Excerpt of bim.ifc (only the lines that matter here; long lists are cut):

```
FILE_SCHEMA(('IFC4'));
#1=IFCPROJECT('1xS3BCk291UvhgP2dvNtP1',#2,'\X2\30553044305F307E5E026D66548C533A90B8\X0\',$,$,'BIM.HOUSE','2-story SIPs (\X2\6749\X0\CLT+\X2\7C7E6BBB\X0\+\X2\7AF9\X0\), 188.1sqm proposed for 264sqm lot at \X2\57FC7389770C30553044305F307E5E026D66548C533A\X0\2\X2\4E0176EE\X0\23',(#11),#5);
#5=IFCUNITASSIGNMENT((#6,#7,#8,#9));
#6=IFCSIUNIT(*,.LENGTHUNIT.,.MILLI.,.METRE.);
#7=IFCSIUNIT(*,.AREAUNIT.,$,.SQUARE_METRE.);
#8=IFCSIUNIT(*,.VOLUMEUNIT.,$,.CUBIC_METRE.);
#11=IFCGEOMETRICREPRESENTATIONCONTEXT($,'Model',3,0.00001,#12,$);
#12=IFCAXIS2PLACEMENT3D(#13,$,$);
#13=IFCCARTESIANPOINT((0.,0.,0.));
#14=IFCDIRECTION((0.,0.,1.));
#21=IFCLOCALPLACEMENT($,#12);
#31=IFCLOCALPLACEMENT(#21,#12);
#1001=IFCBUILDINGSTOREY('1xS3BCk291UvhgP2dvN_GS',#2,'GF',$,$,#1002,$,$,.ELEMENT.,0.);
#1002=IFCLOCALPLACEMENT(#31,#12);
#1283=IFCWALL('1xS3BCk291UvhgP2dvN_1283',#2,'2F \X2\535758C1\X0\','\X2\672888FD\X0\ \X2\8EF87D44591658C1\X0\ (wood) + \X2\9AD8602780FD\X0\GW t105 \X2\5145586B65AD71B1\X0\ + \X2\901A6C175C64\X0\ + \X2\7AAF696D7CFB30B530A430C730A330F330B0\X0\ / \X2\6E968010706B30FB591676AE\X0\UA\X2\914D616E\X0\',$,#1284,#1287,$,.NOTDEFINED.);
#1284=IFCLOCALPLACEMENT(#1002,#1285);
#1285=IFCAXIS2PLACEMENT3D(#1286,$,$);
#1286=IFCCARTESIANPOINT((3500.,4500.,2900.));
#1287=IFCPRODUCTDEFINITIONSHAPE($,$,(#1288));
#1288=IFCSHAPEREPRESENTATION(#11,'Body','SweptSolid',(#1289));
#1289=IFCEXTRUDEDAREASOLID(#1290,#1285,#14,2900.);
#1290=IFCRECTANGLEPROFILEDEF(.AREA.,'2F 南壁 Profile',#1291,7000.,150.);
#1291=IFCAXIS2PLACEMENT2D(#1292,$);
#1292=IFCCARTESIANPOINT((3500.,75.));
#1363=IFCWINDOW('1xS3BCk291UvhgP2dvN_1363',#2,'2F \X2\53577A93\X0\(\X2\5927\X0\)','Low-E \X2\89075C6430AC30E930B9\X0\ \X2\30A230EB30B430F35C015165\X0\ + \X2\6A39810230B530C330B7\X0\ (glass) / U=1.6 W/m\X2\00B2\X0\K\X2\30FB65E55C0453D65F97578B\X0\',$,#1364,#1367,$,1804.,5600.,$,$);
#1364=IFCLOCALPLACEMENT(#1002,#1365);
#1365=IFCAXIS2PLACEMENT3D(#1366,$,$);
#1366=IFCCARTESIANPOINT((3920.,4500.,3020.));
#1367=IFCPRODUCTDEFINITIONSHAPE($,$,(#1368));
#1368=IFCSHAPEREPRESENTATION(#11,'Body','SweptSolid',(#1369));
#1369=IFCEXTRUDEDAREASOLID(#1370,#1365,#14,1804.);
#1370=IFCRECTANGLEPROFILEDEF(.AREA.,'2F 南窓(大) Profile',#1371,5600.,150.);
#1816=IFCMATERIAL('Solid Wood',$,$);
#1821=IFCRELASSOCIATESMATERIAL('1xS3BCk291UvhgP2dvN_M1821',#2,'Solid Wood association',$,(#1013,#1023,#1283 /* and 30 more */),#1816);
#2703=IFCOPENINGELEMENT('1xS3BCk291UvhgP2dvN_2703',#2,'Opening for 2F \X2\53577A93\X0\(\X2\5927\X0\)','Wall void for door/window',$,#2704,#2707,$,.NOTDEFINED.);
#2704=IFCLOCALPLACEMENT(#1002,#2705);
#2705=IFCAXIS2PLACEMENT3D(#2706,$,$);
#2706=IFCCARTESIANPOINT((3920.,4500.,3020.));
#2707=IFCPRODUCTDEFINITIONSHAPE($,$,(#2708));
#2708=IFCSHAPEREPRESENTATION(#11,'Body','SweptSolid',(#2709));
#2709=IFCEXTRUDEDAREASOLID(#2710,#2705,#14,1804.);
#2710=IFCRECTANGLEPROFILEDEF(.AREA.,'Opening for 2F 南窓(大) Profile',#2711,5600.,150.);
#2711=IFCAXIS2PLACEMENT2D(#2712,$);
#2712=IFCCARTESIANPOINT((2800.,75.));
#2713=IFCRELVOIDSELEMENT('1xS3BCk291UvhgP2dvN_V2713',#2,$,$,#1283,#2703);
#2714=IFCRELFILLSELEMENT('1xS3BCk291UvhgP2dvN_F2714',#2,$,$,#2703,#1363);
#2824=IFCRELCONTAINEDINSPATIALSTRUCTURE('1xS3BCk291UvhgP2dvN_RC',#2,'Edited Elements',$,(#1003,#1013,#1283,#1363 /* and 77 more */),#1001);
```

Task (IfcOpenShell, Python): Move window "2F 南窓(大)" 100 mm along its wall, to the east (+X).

```python
import ifcopenshell
import ifcopenshell.api.geometry
import ifcopenshell.util.placement
import ifcopenshell.util.unit

model = ifcopenshell.open("bim.ifc")
unit_scale = ifcopenshell.util.unit.calculate_unit_scale(model)

window = model.by_guid("1xS3BCk291UvhgP2dvN_1363")
opening = window.FillsVoids[0].RelatingOpeningElement
wall = opening.VoidsElements[0].RelatingBuildingElement

wall_matrix = ifcopenshell.util.placement.get_local_placement(wall.ObjectPlacement)
shift = wall_matrix[:3, 0] * 0.1 / unit_scale
before = ifcopenshell.util.placement.get_local_placement(window.ObjectPlacement)[:3, 3].copy()

# The window is not placed relative to its opening, so move both.
for product in (opening, window):
    matrix = ifcopenshell.util.placement.get_local_placement(product.ObjectPlacement)
    matrix[:3, 3] += shift
    ifcopenshell.api.geometry.edit_object_placement(model, product=product, matrix=matrix, is_si=False)

after = ifcopenshell.util.placement.get_local_placement(window.ObjectPlacement)[:3, 3]
print("window moved by", (after - before).round(3) + 0.0)

model.write("bim_edited.ifc")
```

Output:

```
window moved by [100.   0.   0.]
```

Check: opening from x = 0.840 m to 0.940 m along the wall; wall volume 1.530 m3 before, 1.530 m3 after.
